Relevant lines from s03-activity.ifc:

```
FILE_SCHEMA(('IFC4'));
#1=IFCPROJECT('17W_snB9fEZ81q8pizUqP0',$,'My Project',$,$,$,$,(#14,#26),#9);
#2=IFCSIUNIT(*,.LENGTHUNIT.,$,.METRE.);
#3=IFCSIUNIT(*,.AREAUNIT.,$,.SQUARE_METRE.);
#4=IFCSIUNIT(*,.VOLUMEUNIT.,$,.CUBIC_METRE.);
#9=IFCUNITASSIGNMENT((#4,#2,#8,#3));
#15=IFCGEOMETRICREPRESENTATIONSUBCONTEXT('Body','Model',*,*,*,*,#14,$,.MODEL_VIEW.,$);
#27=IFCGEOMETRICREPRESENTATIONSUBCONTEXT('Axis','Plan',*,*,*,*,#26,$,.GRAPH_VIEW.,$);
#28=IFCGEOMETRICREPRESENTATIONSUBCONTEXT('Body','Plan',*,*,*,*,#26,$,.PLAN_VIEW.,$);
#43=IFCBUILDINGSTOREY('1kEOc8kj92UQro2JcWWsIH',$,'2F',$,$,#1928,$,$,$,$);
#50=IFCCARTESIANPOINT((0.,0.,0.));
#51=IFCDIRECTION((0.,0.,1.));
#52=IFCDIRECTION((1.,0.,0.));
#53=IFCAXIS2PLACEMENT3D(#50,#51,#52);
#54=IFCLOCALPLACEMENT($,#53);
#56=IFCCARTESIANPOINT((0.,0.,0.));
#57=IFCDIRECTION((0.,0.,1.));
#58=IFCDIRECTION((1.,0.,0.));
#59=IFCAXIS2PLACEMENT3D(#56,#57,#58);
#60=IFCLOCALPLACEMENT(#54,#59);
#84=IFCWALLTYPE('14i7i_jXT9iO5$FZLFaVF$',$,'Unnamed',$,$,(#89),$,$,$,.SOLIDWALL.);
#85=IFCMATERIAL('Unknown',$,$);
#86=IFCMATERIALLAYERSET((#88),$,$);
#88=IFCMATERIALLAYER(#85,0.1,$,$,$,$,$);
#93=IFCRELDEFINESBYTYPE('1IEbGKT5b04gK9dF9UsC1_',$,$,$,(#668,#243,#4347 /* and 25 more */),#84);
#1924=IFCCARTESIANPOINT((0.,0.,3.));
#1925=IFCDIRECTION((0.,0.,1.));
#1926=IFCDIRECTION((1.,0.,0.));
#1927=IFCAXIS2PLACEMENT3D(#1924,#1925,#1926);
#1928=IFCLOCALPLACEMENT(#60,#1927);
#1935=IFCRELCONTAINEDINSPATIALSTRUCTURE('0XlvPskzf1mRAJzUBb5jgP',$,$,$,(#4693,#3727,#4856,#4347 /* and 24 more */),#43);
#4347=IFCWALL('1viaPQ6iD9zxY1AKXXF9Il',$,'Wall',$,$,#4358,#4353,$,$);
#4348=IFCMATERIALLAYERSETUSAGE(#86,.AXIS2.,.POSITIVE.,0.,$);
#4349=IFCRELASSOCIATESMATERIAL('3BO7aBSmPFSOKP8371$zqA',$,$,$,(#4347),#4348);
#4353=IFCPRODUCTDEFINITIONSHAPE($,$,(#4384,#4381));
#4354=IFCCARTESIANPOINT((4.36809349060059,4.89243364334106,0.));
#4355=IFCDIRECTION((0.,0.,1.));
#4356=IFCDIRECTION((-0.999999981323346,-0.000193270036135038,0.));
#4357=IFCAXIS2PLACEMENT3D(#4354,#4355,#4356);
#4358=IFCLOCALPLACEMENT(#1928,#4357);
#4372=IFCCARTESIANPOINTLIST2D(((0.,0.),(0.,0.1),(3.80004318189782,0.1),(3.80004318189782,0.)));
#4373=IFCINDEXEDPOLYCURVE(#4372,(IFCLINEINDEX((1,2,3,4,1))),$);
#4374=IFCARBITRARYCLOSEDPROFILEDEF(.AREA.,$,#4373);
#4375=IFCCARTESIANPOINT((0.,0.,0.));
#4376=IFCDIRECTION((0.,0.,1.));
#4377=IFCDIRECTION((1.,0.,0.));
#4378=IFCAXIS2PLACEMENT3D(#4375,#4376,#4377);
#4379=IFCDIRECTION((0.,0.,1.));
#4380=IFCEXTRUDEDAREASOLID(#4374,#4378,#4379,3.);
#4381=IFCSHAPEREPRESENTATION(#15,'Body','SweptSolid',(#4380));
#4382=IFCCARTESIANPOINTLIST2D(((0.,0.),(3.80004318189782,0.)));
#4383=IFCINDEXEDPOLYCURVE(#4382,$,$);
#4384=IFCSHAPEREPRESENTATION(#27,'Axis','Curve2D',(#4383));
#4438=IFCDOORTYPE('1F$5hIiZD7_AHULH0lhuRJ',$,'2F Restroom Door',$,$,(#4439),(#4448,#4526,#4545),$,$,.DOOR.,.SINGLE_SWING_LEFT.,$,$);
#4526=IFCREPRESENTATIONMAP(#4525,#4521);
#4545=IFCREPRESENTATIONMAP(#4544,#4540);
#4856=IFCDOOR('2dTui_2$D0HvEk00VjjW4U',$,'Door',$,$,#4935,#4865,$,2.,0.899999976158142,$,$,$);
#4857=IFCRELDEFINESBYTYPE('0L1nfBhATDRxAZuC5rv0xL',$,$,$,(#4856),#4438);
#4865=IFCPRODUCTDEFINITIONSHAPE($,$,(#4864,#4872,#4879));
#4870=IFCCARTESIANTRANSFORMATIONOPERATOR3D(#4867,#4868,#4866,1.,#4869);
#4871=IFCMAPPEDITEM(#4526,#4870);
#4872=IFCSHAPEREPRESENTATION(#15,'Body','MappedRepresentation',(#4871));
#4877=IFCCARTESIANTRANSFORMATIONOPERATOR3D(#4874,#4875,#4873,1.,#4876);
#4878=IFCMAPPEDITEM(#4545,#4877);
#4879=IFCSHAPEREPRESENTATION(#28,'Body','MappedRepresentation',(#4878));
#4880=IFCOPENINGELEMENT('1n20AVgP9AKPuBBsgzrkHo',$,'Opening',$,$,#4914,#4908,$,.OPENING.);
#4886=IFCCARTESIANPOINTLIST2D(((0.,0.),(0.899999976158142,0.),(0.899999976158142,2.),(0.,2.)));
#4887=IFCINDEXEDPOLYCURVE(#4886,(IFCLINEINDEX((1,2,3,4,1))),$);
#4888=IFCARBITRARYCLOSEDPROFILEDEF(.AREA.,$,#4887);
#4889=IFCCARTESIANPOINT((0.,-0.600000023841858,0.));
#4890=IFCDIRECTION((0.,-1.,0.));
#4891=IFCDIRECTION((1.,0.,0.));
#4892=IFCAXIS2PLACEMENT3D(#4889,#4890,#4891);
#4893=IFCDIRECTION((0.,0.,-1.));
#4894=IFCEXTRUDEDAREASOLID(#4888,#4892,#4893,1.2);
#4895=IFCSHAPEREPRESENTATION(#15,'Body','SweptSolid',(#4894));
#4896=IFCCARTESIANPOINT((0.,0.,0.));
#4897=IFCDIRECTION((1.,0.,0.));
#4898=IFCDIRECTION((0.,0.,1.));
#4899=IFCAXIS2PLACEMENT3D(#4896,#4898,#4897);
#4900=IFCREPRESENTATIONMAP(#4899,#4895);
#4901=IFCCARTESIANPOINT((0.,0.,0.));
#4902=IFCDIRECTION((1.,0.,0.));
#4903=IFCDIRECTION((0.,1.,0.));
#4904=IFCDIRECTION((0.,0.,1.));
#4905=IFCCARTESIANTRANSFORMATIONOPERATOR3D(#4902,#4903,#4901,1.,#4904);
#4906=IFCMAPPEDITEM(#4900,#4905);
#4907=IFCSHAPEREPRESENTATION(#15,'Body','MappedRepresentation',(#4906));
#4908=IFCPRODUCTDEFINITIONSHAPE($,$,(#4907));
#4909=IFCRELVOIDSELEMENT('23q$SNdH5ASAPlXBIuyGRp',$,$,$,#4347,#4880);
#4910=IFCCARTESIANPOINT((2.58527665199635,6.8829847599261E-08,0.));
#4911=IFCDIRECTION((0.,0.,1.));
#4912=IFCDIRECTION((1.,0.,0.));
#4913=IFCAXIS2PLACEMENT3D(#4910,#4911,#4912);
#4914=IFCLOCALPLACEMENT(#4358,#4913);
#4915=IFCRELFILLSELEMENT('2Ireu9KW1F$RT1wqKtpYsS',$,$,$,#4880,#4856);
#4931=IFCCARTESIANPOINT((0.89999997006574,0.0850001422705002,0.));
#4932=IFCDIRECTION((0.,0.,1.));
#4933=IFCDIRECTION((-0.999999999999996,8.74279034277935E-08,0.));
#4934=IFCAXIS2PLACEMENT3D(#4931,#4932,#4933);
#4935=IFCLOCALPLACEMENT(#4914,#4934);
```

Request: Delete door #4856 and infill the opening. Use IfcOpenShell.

```python
import ifcopenshell
import ifcopenshell.api.feature
import ifcopenshell.api.root
import ifcopenshell.geom
import ifcopenshell.util.shape

model = ifcopenshell.open("s03-activity.ifc")
settings = ifcopenshell.geom.settings()


def volume(element):
    """Net volume in cubic metres, openings subtracted."""
    shape = ifcopenshell.geom.create_shape(settings, element)
    return ifcopenshell.util.shape.get_volume(shape.geometry)


door = model.by_id(4856)
opening = door.FillsVoids[0].RelatingOpeningElement
wall = opening.VoidsElements[0].RelatingBuildingElement
before = volume(wall)

ifcopenshell.api.root.remove_product(model, product=door)
ifcopenshell.api.feature.remove_feature(model, feature=opening)

after = volume(wall)

print(f"wall volume {before:.3f} -> {after:.3f} m3")

model.write("s03-activity_rev.ifc")
```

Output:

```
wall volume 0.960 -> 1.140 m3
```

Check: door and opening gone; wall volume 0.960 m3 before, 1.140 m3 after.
